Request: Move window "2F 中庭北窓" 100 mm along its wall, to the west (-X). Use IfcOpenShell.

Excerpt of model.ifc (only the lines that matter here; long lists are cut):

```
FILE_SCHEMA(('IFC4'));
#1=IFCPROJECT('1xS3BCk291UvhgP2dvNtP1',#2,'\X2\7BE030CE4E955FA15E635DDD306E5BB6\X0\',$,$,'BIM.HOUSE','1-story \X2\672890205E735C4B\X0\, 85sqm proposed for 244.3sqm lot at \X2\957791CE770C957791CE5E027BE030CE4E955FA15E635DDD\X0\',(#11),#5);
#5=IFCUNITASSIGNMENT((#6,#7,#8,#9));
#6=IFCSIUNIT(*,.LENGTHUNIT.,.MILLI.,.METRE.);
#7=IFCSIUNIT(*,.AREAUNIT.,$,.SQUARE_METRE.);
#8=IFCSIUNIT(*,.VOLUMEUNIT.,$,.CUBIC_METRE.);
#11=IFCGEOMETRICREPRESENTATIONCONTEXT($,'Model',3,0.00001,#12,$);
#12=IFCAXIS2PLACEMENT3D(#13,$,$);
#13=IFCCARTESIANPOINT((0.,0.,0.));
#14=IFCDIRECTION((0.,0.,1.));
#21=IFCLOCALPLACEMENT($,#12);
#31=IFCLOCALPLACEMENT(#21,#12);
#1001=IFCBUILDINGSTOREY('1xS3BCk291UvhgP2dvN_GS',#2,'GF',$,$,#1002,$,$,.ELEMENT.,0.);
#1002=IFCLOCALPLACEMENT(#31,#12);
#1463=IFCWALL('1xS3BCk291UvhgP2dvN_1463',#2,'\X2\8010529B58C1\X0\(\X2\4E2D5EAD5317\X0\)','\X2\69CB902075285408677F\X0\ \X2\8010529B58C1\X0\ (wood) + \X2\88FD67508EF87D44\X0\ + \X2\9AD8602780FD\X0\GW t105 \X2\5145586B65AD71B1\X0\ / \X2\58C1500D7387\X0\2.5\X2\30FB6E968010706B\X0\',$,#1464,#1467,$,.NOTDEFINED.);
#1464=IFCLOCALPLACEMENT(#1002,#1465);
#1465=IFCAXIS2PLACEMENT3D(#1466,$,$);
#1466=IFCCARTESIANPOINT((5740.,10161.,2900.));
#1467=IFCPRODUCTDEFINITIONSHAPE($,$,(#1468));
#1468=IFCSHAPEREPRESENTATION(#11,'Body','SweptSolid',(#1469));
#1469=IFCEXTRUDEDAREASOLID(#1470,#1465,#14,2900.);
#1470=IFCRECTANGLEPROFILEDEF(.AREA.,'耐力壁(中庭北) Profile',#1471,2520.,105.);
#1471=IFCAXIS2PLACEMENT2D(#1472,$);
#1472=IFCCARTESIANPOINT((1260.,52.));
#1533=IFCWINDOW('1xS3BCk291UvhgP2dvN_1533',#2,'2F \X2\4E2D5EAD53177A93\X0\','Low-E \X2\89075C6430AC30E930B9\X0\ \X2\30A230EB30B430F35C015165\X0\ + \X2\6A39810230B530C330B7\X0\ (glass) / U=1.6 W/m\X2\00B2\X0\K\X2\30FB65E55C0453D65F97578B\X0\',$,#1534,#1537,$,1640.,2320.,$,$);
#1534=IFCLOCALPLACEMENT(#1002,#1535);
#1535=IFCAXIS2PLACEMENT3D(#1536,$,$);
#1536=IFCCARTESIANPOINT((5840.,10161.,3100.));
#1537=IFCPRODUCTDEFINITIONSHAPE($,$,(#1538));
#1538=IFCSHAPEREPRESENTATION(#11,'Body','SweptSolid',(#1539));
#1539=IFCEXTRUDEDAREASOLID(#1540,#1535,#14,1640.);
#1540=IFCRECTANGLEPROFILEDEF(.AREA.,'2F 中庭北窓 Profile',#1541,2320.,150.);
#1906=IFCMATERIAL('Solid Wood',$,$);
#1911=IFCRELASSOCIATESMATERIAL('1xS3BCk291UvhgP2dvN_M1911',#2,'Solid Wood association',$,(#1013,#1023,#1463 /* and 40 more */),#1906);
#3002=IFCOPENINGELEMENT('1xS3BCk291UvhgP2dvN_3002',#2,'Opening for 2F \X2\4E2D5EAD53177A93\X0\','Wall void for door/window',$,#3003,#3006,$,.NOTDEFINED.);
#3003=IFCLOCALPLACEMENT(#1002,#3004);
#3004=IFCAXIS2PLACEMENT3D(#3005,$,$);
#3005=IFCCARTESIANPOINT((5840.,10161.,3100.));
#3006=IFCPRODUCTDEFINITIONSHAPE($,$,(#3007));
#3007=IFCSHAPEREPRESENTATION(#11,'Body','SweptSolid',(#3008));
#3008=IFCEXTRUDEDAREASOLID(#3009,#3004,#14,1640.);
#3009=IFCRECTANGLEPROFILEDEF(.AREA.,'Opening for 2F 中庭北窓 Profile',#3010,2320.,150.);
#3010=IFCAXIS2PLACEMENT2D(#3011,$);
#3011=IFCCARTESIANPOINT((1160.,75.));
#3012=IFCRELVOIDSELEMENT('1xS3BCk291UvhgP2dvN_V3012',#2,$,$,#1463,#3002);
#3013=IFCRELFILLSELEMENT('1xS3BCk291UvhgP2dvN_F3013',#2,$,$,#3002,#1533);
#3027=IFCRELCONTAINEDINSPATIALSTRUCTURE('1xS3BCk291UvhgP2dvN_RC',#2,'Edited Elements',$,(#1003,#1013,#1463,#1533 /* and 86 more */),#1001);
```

```python
import ifcopenshell
import ifcopenshell.api.geometry
import ifcopenshell.util.placement

model = ifcopenshell.open("model.ifc")

window = model.by_guid("1xS3BCk291UvhgP2dvN_1533")
opening = window.FillsVoids[0].RelatingOpeningElement
wall = opening.VoidsElements[0].RelatingBuildingElement

wall_matrix = ifcopenshell.util.placement.get_local_placement(wall.ObjectPlacement)
shift = wall_matrix[:3, 0] * -100.0
before = ifcopenshell.util.placement.get_local_placement(window.ObjectPlacement)[:3, 3].copy()

# The window is not placed relative to its opening, so move both.
for product in (opening, window):
    matrix = ifcopenshell.util.placement.get_local_placement(product.ObjectPlacement)
    matrix[:3, 3] += shift
    ifcopenshell.api.geometry.edit_object_placement(model, product=product, matrix=matrix, is_si=False)

after = ifcopenshell.util.placement.get_local_placement(window.ObjectPlacement)[:3, 3]
print("window moved by", (after - before).round(3) + 0.0)

model.write("model_updated.ifc")
```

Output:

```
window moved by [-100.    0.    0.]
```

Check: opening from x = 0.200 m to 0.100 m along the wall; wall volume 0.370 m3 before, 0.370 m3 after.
